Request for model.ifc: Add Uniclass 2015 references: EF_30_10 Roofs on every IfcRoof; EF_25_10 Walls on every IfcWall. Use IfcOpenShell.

First a look at what the model holds.

```python
import ifcopenshell

model = ifcopenshell.open("model.ifc")
print(model.schema)
print("classifications:", [c.Name for c in model.by_type("IfcClassification")])
for ifc_class in ("IfcDoor", "IfcRoof", "IfcStair", "IfcWall", "IfcWindow"):
    print(ifc_class, len(model.by_type(ifc_class)))
```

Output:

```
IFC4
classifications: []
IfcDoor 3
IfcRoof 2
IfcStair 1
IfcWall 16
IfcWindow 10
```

```python
import ifcopenshell
import ifcopenshell.api.classification

model = ifcopenshell.open("model.ifc")

system = ifcopenshell.api.classification.add_classification(model, classification="Uniclass 2015")

codes = {
    "IfcRoof": ("EF_30_10", "Roofs"),
    "IfcWall": ("EF_25_10", "Walls"),
}
for ifc_class, (code, name) in codes.items():
    products = model.by_type(ifc_class)
    ifcopenshell.api.classification.add_reference(
        model, products=products, classification=system, identification=code, name=name
    )
    print(code, len(products))

model.write("model_edited.ifc")
```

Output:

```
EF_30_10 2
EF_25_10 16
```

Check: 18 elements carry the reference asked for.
